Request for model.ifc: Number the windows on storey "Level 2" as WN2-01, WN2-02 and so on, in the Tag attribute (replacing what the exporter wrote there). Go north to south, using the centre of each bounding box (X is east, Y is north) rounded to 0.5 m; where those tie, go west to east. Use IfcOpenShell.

First a look at what the model holds.

```python
import ifcopenshell
import ifcopenshell.util.element
import ifcopenshell.util.placement

model = ifcopenshell.open("model.ifc")
print(model.schema)
storey = next(s for s in model.by_type("IfcBuildingStorey") if s.Name == "Level 2")
windows = [e for e in ifcopenshell.util.element.get_decomposition(storey) if e.is_a("IfcWindow")]
for e in sorted(windows, key=lambda e: e.id()):
    origin = ifcopenshell.util.placement.get_local_placement(e.ObjectPlacement)[:3, 3]
    print(e.id(), e.Tag, e.Name, origin.round(2) + 0.0, sep=" | ")
```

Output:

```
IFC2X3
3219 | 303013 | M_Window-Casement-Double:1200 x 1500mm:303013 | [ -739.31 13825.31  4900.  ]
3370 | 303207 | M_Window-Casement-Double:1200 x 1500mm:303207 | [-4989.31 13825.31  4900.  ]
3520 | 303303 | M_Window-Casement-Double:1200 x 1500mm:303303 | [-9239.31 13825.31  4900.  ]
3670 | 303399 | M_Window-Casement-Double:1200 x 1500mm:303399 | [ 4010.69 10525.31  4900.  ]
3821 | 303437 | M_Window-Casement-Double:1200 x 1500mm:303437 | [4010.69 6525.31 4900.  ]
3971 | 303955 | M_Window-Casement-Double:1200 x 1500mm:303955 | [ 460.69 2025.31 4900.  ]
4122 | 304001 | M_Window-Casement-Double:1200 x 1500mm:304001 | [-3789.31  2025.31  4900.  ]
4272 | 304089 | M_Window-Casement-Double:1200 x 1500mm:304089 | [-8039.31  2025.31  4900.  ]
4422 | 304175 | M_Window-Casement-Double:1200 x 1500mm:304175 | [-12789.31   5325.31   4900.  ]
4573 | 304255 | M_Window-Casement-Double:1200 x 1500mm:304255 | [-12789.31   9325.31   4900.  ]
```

```python
import ifcopenshell
import ifcopenshell.geom
import ifcopenshell.util.element
import ifcopenshell.util.shape

model = ifcopenshell.open("model.ifc")
settings = ifcopenshell.geom.settings()
settings.set("use-world-coords", True)


def centre(element):
    shape = ifcopenshell.geom.create_shape(settings, element)
    return ifcopenshell.util.shape.get_bbox_centroid(shape.geometry)


storey = next(s for s in model.by_type("IfcBuildingStorey") if s.Name == "Level 2")
windows = [e for e in ifcopenshell.util.element.get_decomposition(storey) if e.is_a("IfcWindow")]

# Insertion points can sit at a corner or the storey origin, so sort by the geometry (in metres).
centres = {e: centre(e) for e in windows}
windows.sort(key=lambda e: (-round(centres[e][1] / 0.5), centres[e][0]))

for i, e in enumerate(windows, start=1):
    number = f"WN2-{i:02d}"
    e.Tag = number
    print(e.id(), number)

model.write("model_updated.ifc")
```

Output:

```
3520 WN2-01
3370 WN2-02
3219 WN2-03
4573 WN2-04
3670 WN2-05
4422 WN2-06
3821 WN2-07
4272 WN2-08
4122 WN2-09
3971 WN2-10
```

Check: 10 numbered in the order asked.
